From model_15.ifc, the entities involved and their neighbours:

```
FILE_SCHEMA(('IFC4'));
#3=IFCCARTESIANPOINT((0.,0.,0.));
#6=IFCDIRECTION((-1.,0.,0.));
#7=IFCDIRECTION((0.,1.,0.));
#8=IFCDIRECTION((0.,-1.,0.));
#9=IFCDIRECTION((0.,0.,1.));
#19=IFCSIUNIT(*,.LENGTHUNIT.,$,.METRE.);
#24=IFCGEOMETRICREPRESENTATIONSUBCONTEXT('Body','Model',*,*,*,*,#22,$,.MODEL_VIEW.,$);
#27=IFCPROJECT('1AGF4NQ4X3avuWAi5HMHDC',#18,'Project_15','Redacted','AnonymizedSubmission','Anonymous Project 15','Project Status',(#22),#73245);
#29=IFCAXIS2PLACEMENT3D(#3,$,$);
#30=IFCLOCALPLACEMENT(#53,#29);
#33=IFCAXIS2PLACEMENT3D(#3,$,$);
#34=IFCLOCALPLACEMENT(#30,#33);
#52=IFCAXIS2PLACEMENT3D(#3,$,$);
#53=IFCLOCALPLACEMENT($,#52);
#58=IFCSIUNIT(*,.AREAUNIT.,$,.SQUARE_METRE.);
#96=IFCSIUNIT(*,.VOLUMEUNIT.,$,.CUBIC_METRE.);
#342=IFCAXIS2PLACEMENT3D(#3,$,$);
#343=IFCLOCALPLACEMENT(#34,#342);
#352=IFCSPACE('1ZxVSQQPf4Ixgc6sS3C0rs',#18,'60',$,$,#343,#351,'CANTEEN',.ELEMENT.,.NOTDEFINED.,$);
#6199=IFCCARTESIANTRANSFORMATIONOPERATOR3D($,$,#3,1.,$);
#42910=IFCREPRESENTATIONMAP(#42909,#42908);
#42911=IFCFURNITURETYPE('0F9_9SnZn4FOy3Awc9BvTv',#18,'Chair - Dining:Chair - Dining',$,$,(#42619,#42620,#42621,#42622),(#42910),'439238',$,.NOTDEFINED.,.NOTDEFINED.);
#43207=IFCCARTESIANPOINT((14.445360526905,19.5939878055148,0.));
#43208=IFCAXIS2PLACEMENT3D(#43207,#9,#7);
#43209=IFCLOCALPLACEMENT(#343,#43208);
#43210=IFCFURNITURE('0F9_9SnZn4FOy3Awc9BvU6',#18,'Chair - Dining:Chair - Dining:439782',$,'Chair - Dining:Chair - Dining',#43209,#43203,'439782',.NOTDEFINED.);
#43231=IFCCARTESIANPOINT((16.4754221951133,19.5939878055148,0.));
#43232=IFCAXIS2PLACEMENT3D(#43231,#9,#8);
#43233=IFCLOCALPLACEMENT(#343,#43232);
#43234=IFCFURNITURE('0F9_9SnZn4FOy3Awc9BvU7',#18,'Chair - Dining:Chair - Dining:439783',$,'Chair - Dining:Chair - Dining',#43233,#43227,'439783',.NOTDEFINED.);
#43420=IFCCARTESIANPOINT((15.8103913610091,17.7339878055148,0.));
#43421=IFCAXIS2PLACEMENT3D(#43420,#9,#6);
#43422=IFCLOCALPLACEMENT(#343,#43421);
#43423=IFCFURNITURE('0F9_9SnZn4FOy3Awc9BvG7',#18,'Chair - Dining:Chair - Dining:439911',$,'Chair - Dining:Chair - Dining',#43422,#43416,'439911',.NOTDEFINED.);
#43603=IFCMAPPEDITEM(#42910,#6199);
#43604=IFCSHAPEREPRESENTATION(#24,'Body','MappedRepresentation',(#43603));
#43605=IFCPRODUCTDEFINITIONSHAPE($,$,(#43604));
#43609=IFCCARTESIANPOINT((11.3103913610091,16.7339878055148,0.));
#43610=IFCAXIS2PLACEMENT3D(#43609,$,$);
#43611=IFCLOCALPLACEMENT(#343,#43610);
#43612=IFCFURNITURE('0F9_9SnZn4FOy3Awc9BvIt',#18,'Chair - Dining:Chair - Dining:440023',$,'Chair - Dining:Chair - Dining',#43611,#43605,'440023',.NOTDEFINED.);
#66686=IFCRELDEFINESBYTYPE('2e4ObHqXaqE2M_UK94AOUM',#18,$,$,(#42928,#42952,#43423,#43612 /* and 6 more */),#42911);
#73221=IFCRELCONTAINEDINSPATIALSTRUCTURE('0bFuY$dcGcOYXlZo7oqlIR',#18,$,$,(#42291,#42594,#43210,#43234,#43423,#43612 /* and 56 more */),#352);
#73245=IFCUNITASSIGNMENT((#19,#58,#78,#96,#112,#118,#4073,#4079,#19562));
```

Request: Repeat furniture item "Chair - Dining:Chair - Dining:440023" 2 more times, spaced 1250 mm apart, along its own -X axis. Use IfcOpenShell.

```python
import ifcopenshell
import ifcopenshell.api.geometry
import ifcopenshell.api.root
import ifcopenshell.util.element
import ifcopenshell.util.placement

model = ifcopenshell.open("model_15.ifc")


def reuse_history(source, copy):
    """copy_class also copies each property set's owner history, people and application; keep the originals."""
    for rel in copy.IsDefinedBy:
        if rel.is_a("IfcRelDefinesByProperties") and (history := rel.RelatingPropertyDefinition.OwnerHistory):
            rel.RelatingPropertyDefinition.OwnerHistory = source.OwnerHistory
            ifcopenshell.util.element.remove_deep2(model, history)


source = model.by_id(43612)
base = ifcopenshell.util.placement.get_local_placement(source.ObjectPlacement)
step = -base[:3, 0] * 1.25

for i in range(1, 3):
    copy = ifcopenshell.api.root.copy_class(model, product=source)
    copy.Representation = ifcopenshell.util.element.copy_deep(
        model, source.Representation, exclude=["IfcGeometricRepresentationContext", "IfcRepresentationMap"]
    )
    copy.Name = "Chair - Dining:Chair - Dining"
    copy.Tag = None
    reuse_history(source, copy)
    matrix = base.copy()
    matrix[:3, 3] += i * step
    print("added at", matrix[:3, 3].round(3) + 0.0)
    ifcopenshell.api.geometry.edit_object_placement(model, product=copy, matrix=matrix, is_si=False)

model.write("model_15_updated.ifc")
```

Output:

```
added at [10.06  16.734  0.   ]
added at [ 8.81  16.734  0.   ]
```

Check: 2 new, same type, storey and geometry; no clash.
